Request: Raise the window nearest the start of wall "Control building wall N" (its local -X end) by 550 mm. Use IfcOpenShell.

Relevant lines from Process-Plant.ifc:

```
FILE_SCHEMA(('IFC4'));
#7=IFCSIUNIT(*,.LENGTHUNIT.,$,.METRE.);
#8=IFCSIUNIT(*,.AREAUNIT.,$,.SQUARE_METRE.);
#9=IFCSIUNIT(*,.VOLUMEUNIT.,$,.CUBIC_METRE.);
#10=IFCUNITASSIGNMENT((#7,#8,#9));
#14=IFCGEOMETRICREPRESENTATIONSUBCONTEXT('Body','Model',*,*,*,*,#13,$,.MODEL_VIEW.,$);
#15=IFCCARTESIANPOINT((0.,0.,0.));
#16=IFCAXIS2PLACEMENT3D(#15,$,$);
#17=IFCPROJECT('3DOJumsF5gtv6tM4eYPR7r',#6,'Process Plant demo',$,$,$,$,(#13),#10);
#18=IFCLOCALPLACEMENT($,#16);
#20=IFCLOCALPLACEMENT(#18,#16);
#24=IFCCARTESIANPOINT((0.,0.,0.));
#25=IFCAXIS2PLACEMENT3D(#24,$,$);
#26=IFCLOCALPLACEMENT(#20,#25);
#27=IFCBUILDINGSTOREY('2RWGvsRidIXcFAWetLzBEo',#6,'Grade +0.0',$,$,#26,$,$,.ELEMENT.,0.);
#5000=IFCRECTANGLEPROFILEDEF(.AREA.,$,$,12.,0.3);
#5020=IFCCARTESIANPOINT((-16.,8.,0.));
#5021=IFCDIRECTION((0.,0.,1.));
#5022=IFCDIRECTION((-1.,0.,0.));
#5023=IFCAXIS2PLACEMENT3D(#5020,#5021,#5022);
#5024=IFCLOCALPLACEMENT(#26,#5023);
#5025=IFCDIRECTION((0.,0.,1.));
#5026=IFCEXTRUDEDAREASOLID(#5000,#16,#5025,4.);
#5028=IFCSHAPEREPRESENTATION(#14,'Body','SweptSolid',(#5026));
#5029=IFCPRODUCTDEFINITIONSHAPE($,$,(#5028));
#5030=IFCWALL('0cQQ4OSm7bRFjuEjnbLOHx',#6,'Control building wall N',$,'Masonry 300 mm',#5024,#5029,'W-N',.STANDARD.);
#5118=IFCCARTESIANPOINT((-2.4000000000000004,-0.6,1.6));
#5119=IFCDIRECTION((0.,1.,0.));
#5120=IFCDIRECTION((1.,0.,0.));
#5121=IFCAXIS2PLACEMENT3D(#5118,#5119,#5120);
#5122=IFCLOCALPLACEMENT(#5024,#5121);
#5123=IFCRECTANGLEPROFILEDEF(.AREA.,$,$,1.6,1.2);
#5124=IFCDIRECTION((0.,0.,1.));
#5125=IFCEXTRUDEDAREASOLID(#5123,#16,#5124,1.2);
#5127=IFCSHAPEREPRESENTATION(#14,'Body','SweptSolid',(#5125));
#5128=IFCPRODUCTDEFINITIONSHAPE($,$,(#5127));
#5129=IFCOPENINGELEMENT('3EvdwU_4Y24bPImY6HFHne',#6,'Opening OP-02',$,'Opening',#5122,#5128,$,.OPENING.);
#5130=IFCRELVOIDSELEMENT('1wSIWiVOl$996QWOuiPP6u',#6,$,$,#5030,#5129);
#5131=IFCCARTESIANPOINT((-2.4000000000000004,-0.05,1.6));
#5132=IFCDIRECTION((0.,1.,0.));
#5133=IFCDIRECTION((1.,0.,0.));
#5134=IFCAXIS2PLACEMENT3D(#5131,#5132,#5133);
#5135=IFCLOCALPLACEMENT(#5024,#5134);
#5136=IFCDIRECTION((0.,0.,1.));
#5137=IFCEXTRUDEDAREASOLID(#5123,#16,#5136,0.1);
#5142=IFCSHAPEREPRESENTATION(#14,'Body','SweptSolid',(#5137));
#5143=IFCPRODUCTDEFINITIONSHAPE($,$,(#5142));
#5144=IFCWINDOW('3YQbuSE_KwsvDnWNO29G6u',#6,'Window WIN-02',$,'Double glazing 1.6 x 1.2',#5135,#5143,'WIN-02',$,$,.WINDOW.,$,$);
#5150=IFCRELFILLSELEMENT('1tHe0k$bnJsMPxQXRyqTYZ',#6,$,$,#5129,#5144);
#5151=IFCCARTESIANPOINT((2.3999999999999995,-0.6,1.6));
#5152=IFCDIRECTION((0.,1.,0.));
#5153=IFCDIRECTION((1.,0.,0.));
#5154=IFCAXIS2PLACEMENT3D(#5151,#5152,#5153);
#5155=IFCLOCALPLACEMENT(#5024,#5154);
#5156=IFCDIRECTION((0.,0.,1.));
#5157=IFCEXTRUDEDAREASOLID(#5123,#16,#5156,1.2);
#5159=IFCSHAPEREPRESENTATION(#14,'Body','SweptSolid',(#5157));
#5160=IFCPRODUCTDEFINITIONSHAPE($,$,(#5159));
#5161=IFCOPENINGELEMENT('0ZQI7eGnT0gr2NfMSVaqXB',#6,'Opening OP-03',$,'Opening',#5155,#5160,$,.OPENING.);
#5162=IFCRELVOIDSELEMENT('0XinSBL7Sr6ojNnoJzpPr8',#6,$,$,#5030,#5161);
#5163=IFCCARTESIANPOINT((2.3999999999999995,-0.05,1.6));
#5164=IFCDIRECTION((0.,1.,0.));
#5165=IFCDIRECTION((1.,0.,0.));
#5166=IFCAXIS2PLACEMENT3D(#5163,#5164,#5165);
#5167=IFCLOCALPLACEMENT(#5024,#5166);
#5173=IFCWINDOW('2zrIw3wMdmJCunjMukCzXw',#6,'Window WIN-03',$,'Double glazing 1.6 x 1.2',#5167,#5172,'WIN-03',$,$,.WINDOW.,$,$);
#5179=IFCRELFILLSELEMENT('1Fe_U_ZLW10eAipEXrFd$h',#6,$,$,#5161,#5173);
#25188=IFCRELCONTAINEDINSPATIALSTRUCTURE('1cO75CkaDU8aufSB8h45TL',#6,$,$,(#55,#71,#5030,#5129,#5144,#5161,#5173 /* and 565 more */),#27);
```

```python
import numpy as np
import ifcopenshell
import ifcopenshell.api.geometry
import ifcopenshell.util.placement
import ifcopenshell.util.unit

model = ifcopenshell.open("Process-Plant.ifc")
unit_scale = ifcopenshell.util.unit.calculate_unit_scale(model)

window = model.by_id(5144)
opening = window.FillsVoids[0].RelatingOpeningElement
dz = 0.55

shift = np.array([0.0, 0.0, dz])
# The window is not placed relative to its opening, so move both.
for product in (opening, window):
    matrix = ifcopenshell.util.placement.get_local_placement(product.ObjectPlacement)
    matrix[:3, 3] += shift
    ifcopenshell.api.geometry.edit_object_placement(model, product=product, matrix=matrix, is_si=False)

print(f"moved by {dz * unit_scale:+.3f} m")

model.write("Process-Plant-out.ifc")
```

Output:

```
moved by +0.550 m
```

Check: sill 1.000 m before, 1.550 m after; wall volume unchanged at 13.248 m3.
